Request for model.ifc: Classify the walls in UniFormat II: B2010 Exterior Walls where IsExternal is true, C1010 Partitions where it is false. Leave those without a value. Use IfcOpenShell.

First a look at what the model holds.

```python
import ifcopenshell
import ifcopenshell.util.element

model = ifcopenshell.open("model.ifc")
print(model.schema)
print("classifications:", [c.Name for c in model.by_type("IfcClassification")])
values = [ifcopenshell.util.element.get_pset(e, "Pset_WallCommon", "IsExternal") for e in model.by_type("IfcWall")]
for value in (True, False, None):
    print("IsExternal", value, values.count(value))
```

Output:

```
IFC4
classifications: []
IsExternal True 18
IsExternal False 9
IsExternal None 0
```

```python
import ifcopenshell
import ifcopenshell.api.classification
import ifcopenshell.util.element

model = ifcopenshell.open("model.ifc")

system = ifcopenshell.api.classification.add_classification(model, classification="UniFormat II")

walls = model.by_type("IfcWall")
external = {e: ifcopenshell.util.element.get_pset(e, "Pset_WallCommon", "IsExternal") for e in walls}
for flag, code, name in ((True, "B2010", "Exterior Walls"), (False, "C1010", "Partitions")):
    products = [e for e in walls if external[e] is flag]
    ifcopenshell.api.classification.add_reference(
        model, products=products, classification=system, identification=code, name=name
    )
    print(code, len(products))

model.write("model_updated.ifc")
```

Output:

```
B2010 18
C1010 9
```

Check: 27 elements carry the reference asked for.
